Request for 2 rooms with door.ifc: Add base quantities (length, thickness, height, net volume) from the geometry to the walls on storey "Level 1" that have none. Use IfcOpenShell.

First a look at what the model holds.

```python
import ifcopenshell
import ifcopenshell.util.element
import ifcopenshell.util.unit

model = ifcopenshell.open("2 rooms with door.ifc")
print(model.schema)
for unit_type in ("LENGTHUNIT", "AREAUNIT", "VOLUMEUNIT"):
    print(unit_type, ifcopenshell.util.unit.calculate_unit_scale(model, unit_type))
storey = next(s for s in model.by_type("IfcBuildingStorey") if s.Name == "Level 1")
walls = [e for e in ifcopenshell.util.element.get_decomposition(storey) if e.is_a("IfcWall")]
for e in sorted(walls, key=lambda e: e.id()):
    print(e.id(), e.is_a(), e.Name, list(ifcopenshell.util.element.get_psets(e, qtos_only=True)), sep=" | ")
```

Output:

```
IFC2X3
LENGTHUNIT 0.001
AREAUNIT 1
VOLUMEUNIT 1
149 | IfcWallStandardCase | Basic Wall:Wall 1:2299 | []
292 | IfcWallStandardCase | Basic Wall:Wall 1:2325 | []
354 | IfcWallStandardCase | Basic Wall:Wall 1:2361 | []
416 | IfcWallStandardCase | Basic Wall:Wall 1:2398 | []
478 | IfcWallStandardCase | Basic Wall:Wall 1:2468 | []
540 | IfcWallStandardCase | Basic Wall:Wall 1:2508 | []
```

```python
import ifcopenshell
import ifcopenshell.api.pset
import ifcopenshell.geom
import ifcopenshell.util.element
import ifcopenshell.util.shape
import ifcopenshell.util.unit

model = ifcopenshell.open("2 rooms with door.ifc")
unit_scale = ifcopenshell.util.unit.calculate_unit_scale(model)
volume_scale = ifcopenshell.util.unit.calculate_unit_scale(model, "VOLUMEUNIT")
settings = ifcopenshell.geom.settings()

storey = next(s for s in model.by_type("IfcBuildingStorey") if s.Name == "Level 1")
walls = [e for e in ifcopenshell.util.element.get_decomposition(storey) if e.is_a("IfcWall")]

for e in sorted(walls, key=lambda e: e.id()):
    if ifcopenshell.util.element.get_psets(e, qtos_only=True, should_inherit=False):
        continue
    # Geometry comes back in metres, in the element's own axes.
    shape = ifcopenshell.geom.create_shape(settings, e)
    values = {
        "Length": ifcopenshell.util.shape.get_x(shape.geometry) / unit_scale,
        "Width": ifcopenshell.util.shape.get_y(shape.geometry) / unit_scale,
        "Height": ifcopenshell.util.shape.get_z(shape.geometry) / unit_scale,
        "NetVolume": ifcopenshell.util.shape.get_volume(shape.geometry) / volume_scale,
    }
    qto = ifcopenshell.api.pset.add_qto(model, product=e, name="BaseQuantities")
    ifcopenshell.api.pset.edit_qto(model, qto=qto, properties=values)
    print(e.id(), {k: round(v, 3) for k, v in values.items()})

model.write("2 rooms with door_updated.ifc")
```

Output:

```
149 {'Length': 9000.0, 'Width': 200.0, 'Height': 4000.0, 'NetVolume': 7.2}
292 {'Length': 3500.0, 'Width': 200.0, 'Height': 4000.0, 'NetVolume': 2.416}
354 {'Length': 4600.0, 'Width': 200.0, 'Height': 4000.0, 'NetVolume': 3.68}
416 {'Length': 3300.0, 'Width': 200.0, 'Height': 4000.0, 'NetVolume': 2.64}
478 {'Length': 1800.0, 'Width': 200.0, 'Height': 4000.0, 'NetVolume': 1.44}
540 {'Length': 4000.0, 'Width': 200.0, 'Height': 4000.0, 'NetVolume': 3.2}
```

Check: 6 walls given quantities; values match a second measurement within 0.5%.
